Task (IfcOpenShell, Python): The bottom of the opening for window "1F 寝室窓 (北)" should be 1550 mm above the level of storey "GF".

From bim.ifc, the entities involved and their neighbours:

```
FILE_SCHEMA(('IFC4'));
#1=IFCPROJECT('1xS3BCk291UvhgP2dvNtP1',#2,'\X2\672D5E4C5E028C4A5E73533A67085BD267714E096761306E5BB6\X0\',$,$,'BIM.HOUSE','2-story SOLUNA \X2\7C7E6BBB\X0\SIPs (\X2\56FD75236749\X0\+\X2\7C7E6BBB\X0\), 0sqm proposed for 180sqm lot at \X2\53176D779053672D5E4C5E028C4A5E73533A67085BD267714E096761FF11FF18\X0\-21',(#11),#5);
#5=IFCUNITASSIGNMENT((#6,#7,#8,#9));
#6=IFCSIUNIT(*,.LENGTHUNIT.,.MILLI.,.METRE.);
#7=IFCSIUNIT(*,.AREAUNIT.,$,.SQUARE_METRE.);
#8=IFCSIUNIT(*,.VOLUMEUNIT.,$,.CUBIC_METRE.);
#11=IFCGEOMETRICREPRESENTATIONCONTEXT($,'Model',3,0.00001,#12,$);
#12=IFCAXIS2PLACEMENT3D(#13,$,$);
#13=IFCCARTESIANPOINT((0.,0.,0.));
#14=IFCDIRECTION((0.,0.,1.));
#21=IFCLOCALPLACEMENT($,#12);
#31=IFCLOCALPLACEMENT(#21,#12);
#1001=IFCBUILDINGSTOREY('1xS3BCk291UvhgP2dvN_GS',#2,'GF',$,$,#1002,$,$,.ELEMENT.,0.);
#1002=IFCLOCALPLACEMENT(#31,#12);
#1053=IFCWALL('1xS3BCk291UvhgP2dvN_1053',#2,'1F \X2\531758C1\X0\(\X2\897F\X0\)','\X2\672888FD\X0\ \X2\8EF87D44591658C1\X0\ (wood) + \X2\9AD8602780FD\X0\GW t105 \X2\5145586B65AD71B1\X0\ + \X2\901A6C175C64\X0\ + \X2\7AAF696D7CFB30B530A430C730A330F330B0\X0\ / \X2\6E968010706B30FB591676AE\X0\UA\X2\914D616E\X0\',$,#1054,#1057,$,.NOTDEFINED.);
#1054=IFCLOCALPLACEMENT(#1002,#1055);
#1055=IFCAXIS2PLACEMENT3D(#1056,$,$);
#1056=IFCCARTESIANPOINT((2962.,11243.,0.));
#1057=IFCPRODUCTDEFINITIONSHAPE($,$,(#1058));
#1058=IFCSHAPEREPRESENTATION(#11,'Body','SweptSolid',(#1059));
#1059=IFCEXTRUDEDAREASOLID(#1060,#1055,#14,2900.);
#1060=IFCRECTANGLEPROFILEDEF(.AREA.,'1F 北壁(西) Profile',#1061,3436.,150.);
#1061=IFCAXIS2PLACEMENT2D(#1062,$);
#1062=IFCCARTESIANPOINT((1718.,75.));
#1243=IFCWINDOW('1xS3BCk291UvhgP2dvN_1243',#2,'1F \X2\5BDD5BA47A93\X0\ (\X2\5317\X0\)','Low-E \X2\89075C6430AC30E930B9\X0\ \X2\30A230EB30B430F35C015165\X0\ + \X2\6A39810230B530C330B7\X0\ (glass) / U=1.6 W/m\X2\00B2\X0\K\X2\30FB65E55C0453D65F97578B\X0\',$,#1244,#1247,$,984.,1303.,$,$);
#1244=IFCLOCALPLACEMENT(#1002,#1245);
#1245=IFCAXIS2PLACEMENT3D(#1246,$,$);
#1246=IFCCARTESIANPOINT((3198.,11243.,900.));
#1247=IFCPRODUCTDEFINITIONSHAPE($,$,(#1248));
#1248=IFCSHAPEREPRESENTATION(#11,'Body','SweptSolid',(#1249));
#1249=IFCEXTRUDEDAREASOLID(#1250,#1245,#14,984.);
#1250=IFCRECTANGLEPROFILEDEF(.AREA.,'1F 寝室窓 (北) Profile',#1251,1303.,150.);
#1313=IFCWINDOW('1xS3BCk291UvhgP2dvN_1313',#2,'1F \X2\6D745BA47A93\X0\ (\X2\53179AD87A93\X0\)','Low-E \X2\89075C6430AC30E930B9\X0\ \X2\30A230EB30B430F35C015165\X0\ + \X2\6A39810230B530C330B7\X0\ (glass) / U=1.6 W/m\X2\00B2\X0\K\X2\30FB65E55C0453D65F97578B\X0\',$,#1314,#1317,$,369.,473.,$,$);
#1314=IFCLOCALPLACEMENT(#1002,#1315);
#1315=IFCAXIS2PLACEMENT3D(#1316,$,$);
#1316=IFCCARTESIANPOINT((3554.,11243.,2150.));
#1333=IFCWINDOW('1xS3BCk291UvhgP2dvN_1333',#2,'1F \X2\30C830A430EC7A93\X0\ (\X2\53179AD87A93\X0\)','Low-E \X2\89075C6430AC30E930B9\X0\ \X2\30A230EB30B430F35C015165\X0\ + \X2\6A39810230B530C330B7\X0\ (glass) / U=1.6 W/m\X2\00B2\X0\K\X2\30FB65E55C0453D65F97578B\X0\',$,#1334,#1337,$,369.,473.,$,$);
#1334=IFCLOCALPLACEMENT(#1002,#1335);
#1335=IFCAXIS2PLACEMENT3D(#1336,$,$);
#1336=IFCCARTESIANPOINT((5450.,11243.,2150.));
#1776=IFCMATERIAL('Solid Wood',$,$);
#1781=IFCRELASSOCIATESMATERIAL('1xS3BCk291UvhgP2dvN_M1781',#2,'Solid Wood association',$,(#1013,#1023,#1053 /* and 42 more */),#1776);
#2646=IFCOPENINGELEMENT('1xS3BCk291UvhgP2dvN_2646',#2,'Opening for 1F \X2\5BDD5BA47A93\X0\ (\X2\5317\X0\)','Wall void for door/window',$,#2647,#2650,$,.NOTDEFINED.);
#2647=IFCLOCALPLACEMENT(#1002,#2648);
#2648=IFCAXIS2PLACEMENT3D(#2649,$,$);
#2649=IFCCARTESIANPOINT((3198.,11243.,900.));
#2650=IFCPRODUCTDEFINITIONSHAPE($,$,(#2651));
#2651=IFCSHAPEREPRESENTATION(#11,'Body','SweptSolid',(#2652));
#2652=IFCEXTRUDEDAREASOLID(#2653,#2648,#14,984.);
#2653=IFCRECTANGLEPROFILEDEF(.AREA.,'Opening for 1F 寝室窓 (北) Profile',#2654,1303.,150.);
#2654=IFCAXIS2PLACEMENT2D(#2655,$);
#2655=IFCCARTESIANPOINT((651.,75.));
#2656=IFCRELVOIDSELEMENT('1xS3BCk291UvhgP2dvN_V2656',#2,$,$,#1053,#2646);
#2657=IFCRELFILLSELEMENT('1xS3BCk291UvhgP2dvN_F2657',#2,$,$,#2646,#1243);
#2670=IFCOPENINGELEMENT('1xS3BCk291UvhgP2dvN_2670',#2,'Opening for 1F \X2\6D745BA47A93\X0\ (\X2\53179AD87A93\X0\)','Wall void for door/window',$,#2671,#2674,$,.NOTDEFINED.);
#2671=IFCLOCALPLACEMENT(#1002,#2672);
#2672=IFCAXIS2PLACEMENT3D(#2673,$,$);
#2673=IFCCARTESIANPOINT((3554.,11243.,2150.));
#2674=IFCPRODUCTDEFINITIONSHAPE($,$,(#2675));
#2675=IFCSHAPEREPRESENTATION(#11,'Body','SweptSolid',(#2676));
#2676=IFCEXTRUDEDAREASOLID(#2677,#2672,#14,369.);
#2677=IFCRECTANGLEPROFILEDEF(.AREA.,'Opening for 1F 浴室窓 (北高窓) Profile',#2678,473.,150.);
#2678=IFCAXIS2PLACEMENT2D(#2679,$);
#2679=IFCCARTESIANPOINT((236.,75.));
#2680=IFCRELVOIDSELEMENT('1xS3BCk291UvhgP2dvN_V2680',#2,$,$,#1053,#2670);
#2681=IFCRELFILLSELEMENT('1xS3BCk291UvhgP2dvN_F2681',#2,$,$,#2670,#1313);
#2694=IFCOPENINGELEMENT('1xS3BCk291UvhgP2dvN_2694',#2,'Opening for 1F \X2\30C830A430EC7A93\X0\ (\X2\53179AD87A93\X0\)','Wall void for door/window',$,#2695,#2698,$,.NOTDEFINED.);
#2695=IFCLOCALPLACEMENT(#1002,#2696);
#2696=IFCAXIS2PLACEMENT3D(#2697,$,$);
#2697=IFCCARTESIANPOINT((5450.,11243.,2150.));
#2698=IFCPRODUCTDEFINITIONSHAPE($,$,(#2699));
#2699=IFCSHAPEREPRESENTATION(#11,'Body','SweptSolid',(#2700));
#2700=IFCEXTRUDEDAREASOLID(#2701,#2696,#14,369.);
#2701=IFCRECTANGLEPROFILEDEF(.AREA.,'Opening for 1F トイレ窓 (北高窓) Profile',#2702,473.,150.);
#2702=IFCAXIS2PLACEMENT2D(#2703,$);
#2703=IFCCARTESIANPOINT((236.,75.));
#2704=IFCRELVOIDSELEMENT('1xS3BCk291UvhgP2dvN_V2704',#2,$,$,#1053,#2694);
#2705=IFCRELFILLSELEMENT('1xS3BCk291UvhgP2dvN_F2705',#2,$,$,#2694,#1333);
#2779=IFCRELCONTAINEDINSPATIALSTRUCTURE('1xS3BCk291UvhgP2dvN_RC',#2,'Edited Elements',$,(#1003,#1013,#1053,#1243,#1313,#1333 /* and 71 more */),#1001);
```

```python
import numpy as np
import ifcopenshell
import ifcopenshell.api.geometry
import ifcopenshell.geom
import ifcopenshell.util.element
import ifcopenshell.util.placement
import ifcopenshell.util.shape
import ifcopenshell.util.unit

model = ifcopenshell.open("bim.ifc")
unit_scale = ifcopenshell.util.unit.calculate_unit_scale(model)

window = model.by_id(1243)
opening = window.FillsVoids[0].RelatingOpeningElement
storey = ifcopenshell.util.element.get_container(window, ifc_class="IfcBuildingStorey")
level = ifcopenshell.util.placement.get_local_placement(storey.ObjectPlacement)[2, 3]

# The opening's origin need not be at the sill, so measure its lowest point.
shape = ifcopenshell.geom.create_shape(ifcopenshell.geom.settings(), opening)
bottom = ifcopenshell.util.shape.get_shape_bottom_elevation(shape, shape.geometry) / unit_scale
dz = level + 1550.0 - bottom

shift = np.array([0.0, 0.0, dz])
# The window is not placed relative to its opening, so move both.
for product in (opening, window):
    matrix = ifcopenshell.util.placement.get_local_placement(product.ObjectPlacement)
    matrix[:3, 3] += shift
    ifcopenshell.api.geometry.edit_object_placement(model, product=product, matrix=matrix, is_si=False)

print(f"moved by {dz * unit_scale:+.3f} m")

model.write("bim_edited.ifc")
```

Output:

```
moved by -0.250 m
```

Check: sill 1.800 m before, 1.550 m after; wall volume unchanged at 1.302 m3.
